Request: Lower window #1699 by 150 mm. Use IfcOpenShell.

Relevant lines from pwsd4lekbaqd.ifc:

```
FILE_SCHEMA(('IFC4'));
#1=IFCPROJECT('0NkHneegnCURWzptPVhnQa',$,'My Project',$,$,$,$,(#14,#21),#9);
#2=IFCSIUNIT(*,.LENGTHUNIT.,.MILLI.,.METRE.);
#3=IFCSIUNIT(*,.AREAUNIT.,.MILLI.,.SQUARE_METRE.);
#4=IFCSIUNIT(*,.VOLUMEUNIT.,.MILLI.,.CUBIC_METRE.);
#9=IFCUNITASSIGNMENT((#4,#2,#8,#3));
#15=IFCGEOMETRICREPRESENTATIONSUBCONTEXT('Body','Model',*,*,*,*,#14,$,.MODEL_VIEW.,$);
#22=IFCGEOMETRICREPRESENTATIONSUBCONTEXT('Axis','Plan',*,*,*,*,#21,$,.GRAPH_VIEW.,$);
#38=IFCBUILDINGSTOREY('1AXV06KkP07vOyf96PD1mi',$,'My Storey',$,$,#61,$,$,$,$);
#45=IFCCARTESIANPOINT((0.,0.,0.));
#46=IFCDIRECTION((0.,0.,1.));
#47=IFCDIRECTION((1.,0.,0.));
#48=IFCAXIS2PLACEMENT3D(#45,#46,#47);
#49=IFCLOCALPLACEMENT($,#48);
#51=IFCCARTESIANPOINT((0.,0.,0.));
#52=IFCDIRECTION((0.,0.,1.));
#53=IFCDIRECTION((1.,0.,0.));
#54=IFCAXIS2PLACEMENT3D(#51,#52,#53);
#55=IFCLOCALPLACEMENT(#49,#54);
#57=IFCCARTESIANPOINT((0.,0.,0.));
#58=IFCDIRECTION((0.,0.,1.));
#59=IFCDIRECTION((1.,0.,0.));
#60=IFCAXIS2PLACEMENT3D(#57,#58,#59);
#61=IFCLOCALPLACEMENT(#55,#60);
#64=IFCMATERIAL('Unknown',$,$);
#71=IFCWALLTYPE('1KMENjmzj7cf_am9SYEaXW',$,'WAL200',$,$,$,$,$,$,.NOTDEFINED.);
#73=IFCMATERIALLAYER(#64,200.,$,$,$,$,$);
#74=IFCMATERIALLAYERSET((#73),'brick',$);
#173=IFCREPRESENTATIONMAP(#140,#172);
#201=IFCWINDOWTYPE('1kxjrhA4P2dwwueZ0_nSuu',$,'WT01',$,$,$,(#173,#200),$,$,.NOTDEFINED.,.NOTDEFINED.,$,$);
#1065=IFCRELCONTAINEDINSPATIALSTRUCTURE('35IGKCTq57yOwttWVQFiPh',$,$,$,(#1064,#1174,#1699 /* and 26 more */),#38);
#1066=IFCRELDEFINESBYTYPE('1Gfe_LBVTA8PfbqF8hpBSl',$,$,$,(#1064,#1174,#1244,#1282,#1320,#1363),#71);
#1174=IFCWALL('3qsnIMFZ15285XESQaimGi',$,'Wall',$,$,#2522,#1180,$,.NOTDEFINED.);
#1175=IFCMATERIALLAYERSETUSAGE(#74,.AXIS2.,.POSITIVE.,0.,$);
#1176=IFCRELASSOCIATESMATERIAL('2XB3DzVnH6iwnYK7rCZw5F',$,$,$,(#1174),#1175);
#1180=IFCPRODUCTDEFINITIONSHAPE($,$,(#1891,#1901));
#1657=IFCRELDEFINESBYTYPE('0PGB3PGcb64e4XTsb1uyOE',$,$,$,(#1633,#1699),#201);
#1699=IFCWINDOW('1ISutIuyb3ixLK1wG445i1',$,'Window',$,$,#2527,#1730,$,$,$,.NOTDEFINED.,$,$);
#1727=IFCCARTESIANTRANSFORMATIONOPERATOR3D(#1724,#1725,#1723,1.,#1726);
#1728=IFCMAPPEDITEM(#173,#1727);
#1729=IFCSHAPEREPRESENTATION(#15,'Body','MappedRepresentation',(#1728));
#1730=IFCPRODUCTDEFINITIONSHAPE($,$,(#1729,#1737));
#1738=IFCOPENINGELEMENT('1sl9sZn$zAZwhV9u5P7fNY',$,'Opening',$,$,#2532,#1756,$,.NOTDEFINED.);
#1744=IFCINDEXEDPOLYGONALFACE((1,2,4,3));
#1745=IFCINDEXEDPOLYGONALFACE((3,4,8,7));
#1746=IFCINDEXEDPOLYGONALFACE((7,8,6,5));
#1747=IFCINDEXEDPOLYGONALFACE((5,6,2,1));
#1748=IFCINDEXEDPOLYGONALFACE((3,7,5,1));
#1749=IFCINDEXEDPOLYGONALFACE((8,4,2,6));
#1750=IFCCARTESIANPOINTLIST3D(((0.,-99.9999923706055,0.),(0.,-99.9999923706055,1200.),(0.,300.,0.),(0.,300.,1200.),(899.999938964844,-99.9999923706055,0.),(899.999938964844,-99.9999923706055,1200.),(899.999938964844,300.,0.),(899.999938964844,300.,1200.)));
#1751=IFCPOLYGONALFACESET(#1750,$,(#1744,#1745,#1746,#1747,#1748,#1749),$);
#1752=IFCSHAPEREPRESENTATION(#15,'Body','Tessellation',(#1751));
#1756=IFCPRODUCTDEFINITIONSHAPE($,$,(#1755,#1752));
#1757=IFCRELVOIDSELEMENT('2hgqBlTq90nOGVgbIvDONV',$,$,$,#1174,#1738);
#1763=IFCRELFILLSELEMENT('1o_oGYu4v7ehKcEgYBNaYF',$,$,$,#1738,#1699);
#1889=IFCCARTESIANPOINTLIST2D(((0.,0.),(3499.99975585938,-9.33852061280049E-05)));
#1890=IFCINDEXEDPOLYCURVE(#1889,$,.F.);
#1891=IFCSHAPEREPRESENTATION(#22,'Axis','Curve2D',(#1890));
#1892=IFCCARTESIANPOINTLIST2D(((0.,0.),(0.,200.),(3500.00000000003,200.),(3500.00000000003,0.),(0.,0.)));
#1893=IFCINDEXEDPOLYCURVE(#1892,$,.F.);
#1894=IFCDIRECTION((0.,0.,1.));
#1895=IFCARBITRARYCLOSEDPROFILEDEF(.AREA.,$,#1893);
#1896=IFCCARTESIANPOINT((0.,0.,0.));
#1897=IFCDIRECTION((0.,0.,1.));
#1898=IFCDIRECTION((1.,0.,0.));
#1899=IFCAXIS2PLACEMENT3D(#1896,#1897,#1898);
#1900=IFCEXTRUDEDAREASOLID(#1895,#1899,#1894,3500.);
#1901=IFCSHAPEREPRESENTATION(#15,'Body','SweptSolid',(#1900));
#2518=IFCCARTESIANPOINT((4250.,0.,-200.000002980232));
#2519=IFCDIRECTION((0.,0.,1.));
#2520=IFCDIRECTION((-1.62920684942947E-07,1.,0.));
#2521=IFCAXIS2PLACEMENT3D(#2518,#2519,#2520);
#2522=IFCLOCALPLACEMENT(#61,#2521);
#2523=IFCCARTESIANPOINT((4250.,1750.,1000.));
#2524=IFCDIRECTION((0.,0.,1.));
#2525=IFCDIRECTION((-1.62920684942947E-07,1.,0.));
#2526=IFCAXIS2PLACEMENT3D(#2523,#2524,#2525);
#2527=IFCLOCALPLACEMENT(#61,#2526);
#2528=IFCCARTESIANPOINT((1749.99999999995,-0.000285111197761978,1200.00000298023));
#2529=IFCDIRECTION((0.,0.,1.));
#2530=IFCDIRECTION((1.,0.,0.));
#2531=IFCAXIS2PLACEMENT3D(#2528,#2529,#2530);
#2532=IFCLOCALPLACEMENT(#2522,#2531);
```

```python
import numpy as np
import ifcopenshell
import ifcopenshell.api.geometry
import ifcopenshell.util.placement
import ifcopenshell.util.unit

model = ifcopenshell.open("pwsd4lekbaqd.ifc")
unit_scale = ifcopenshell.util.unit.calculate_unit_scale(model)

window = model.by_guid("1ISutIuyb3ixLK1wG445i1")
opening = window.FillsVoids[0].RelatingOpeningElement
dz = -150.0

shift = np.array([0.0, 0.0, dz])
# The window is not placed relative to its opening, so move both.
for product in (opening, window):
    matrix = ifcopenshell.util.placement.get_local_placement(product.ObjectPlacement)
    matrix[:3, 3] += shift
    ifcopenshell.api.geometry.edit_object_placement(model, product=product, matrix=matrix, is_si=False)

print(f"moved by {dz * unit_scale:+.3f} m")

model.write("pwsd4lekbaqd_edited.ifc")
```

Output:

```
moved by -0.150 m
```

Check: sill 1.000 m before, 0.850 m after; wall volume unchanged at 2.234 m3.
